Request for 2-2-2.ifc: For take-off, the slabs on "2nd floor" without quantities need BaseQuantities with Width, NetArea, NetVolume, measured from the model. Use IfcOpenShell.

First a look at what the model holds.

```python
import ifcopenshell
import ifcopenshell.util.element
import ifcopenshell.util.unit

model = ifcopenshell.open("2-2-2.ifc")
print(model.schema)
for unit_type in ("LENGTHUNIT", "AREAUNIT", "VOLUMEUNIT"):
    print(unit_type, ifcopenshell.util.unit.calculate_unit_scale(model, unit_type))
storey = next(s for s in model.by_type("IfcBuildingStorey") if s.Name == "2nd floor")
slabs = [e for e in ifcopenshell.util.element.get_decomposition(storey) if e.is_a("IfcSlab")]
for e in sorted(slabs, key=lambda e: e.id()):
    print(e.id(), e.is_a(), e.Name, list(ifcopenshell.util.element.get_psets(e, qtos_only=True)), sep=" | ")
```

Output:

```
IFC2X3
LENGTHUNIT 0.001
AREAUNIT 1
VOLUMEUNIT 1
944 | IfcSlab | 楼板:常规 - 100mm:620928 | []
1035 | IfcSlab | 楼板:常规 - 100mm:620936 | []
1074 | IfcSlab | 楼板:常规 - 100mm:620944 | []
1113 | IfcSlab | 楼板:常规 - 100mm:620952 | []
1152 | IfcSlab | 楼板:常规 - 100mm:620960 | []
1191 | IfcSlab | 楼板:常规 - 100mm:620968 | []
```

```python
import ifcopenshell
import ifcopenshell.api.pset
import ifcopenshell.geom
import ifcopenshell.util.element
import ifcopenshell.util.shape
import ifcopenshell.util.unit

model = ifcopenshell.open("2-2-2.ifc")
unit_scale = ifcopenshell.util.unit.calculate_unit_scale(model)
area_scale = ifcopenshell.util.unit.calculate_unit_scale(model, "AREAUNIT")
volume_scale = ifcopenshell.util.unit.calculate_unit_scale(model, "VOLUMEUNIT")
settings = ifcopenshell.geom.settings()

storey = next(s for s in model.by_type("IfcBuildingStorey") if s.Name == "2nd floor")
slabs = [e for e in ifcopenshell.util.element.get_decomposition(storey) if e.is_a("IfcSlab")]

for e in sorted(slabs, key=lambda e: e.id()):
    if ifcopenshell.util.element.get_psets(e, qtos_only=True, should_inherit=False):
        continue
    # Geometry comes back in metres, in the element's own axes.
    shape = ifcopenshell.geom.create_shape(settings, e)
    values = {
        "Width": ifcopenshell.util.shape.get_z(shape.geometry) / unit_scale,
        "NetArea": ifcopenshell.util.shape.get_footprint_area(shape.geometry) / area_scale,
        "NetVolume": ifcopenshell.util.shape.get_volume(shape.geometry) / volume_scale,
    }
    qto = ifcopenshell.api.pset.add_qto(model, product=e, name="BaseQuantities")
    ifcopenshell.api.pset.edit_qto(model, qto=qto, properties=values)
    print(e.id(), {k: round(v, 3) for k, v in values.items()})

model.write("2-2-2_rev.ifc")
```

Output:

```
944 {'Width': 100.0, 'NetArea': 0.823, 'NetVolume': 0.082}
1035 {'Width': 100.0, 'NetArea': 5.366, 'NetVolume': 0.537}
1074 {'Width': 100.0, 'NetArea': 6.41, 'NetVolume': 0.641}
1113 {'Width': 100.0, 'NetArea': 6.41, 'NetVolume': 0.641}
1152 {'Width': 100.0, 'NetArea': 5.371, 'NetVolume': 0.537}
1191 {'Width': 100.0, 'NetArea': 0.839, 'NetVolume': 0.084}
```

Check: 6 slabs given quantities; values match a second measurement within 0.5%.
